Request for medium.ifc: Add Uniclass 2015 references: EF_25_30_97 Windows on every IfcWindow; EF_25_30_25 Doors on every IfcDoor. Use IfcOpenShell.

First a look at what the model holds.

```python
import ifcopenshell

model = ifcopenshell.open("medium.ifc")
print(model.schema)
print("classifications:", [c.Name for c in model.by_type("IfcClassification")])
for ifc_class in ("IfcDoor", "IfcRoof", "IfcStair", "IfcWall", "IfcWindow"):
    print(ifc_class, len(model.by_type(ifc_class)))
```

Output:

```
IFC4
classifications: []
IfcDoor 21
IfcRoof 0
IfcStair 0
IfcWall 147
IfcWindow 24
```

```python
import ifcopenshell
import ifcopenshell.api.classification

model = ifcopenshell.open("medium.ifc")

system = ifcopenshell.api.classification.add_classification(model, classification="Uniclass 2015")

codes = {
    "IfcWindow": ("EF_25_30_97", "Windows"),
    "IfcDoor": ("EF_25_30_25", "Doors"),
}
for ifc_class, (code, name) in codes.items():
    products = model.by_type(ifc_class)
    ifcopenshell.api.classification.add_reference(
        model, products=products, classification=system, identification=code, name=name
    )
    print(code, len(products))

model.write("medium_rev.ifc")
```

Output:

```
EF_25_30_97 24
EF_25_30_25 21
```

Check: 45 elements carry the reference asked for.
